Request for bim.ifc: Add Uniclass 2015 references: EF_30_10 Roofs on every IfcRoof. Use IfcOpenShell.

First a look at what the model holds.

```python
import ifcopenshell

model = ifcopenshell.open("bim.ifc")
print(model.schema)
print("classifications:", [c.Name for c in model.by_type("IfcClassification")])
for ifc_class in ("IfcDoor", "IfcRoof", "IfcStair", "IfcWall", "IfcWindow"):
    print(ifc_class, len(model.by_type(ifc_class)))
```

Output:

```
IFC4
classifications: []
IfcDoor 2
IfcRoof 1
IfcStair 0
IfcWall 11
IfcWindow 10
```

```python
import ifcopenshell
import ifcopenshell.api.classification

model = ifcopenshell.open("bim.ifc")

system = ifcopenshell.api.classification.add_classification(model, classification="Uniclass 2015")

codes = {
    "IfcRoof": ("EF_30_10", "Roofs"),
}
for ifc_class, (code, name) in codes.items():
    products = model.by_type(ifc_class)
    ifcopenshell.api.classification.add_reference(
        model, products=products, classification=system, identification=code, name=name
    )
    print(code, len(products))

model.write("bim_rev.ifc")
```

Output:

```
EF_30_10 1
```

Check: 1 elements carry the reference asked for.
